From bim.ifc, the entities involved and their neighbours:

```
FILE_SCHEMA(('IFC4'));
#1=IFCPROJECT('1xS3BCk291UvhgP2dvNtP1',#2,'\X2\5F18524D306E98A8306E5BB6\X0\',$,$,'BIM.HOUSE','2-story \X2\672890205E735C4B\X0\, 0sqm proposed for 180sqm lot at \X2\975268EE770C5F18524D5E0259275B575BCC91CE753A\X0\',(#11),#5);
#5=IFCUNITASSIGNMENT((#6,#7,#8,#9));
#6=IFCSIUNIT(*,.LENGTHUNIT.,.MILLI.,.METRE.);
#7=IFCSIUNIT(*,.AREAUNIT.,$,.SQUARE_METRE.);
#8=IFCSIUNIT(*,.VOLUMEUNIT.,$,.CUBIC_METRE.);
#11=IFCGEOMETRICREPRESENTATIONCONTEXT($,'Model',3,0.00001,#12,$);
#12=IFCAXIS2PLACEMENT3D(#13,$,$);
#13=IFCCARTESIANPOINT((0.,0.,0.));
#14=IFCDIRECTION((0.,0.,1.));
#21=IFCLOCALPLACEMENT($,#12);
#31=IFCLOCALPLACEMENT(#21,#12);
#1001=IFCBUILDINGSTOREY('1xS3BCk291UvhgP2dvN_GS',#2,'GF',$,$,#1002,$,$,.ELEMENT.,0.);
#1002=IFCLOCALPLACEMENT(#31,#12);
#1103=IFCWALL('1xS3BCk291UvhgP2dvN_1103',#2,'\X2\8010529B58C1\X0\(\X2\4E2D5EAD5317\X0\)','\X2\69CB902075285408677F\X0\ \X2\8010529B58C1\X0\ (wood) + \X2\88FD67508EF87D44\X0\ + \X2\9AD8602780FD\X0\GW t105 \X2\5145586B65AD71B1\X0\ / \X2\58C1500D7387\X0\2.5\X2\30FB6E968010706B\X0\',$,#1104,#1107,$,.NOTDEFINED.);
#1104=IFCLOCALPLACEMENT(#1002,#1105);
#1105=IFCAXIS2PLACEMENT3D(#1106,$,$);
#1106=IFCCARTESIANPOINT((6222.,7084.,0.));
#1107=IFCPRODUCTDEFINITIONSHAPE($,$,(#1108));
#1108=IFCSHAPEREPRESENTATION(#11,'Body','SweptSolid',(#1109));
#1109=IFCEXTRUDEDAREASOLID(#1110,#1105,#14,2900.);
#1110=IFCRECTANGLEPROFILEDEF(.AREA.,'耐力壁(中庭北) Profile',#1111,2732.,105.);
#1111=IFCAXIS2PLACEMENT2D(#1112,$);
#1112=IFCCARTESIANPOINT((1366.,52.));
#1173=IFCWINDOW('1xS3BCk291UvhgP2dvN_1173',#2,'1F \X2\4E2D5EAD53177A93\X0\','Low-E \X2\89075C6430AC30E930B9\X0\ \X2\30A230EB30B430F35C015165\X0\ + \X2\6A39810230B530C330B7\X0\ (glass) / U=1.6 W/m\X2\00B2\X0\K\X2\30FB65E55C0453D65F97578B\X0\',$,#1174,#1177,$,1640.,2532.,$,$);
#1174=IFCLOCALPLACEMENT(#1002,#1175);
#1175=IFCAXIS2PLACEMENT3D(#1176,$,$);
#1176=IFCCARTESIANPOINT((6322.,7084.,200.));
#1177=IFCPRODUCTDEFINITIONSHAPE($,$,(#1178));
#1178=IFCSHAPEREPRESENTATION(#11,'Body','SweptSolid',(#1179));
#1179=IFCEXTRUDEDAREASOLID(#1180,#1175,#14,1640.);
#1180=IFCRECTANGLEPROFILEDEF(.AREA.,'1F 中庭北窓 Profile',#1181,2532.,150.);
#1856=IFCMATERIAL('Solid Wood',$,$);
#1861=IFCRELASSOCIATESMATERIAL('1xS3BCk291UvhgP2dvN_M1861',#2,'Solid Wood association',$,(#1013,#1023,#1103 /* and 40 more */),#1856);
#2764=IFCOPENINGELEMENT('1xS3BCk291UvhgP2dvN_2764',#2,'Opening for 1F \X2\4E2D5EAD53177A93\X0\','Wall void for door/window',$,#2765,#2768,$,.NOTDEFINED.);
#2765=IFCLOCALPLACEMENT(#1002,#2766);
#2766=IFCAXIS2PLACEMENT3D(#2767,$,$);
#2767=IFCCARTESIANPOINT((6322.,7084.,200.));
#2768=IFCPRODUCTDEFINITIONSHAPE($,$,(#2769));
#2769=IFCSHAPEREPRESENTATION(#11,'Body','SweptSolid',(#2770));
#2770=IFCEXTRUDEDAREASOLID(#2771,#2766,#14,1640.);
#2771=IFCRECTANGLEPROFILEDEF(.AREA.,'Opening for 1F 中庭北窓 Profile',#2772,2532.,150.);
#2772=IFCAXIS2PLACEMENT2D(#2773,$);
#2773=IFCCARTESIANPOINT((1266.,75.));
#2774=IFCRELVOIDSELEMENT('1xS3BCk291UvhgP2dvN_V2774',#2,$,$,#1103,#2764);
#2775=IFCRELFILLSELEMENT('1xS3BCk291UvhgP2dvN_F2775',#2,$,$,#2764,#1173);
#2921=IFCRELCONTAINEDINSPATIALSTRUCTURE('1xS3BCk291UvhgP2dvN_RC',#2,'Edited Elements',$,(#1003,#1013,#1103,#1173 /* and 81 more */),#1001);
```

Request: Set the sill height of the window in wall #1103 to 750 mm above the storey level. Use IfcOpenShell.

```python
import numpy as np
import ifcopenshell
import ifcopenshell.api.geometry
import ifcopenshell.geom
import ifcopenshell.util.element
import ifcopenshell.util.placement
import ifcopenshell.util.shape
import ifcopenshell.util.unit

model = ifcopenshell.open("bim.ifc")
unit_scale = ifcopenshell.util.unit.calculate_unit_scale(model)

window = model.by_guid("1xS3BCk291UvhgP2dvN_1173")
opening = window.FillsVoids[0].RelatingOpeningElement
storey = ifcopenshell.util.element.get_container(window, ifc_class="IfcBuildingStorey")
level = ifcopenshell.util.placement.get_local_placement(storey.ObjectPlacement)[2, 3]

# The opening's origin need not be at the sill, so measure its lowest point.
shape = ifcopenshell.geom.create_shape(ifcopenshell.geom.settings(), opening)
bottom = ifcopenshell.util.shape.get_shape_bottom_elevation(shape, shape.geometry) / unit_scale
dz = level + 0.75 / unit_scale - bottom

shift = np.array([0.0, 0.0, dz])
# The window is not placed relative to its opening, so move both.
for product in (opening, window):
    matrix = ifcopenshell.util.placement.get_local_placement(product.ObjectPlacement)
    matrix[:3, 3] += shift
    ifcopenshell.api.geometry.edit_object_placement(model, product=product, matrix=matrix, is_si=False)

print(f"moved by {dz * unit_scale:+.3f} m")

model.write("bim_rev.ifc")
```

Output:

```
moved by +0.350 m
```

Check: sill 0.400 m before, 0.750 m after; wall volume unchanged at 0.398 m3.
